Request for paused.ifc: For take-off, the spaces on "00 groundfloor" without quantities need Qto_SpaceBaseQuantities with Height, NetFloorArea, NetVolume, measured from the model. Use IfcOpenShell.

First a look at what the model holds.

```python
import ifcopenshell
import ifcopenshell.util.element
import ifcopenshell.util.unit

model = ifcopenshell.open("paused.ifc")
print(model.schema)
for unit_type in ("LENGTHUNIT", "AREAUNIT", "VOLUMEUNIT"):
    print(unit_type, ifcopenshell.util.unit.calculate_unit_scale(model, unit_type))
storey = next(s for s in model.by_type("IfcBuildingStorey") if s.Name == "00 groundfloor")
spaces = [e for e in ifcopenshell.util.element.get_decomposition(storey) if e.is_a("IfcSpace")]
for e in sorted(spaces, key=lambda e: e.id()):
    print(e.id(), e.is_a(), e.Name, list(ifcopenshell.util.element.get_psets(e, qtos_only=True)), sep=" | ")
```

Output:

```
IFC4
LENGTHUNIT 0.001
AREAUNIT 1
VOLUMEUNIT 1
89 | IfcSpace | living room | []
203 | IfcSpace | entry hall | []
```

```python
import ifcopenshell
import ifcopenshell.api.pset
import ifcopenshell.geom
import ifcopenshell.util.element
import ifcopenshell.util.shape
import ifcopenshell.util.unit

model = ifcopenshell.open("paused.ifc")
unit_scale = ifcopenshell.util.unit.calculate_unit_scale(model)
area_scale = ifcopenshell.util.unit.calculate_unit_scale(model, "AREAUNIT")
volume_scale = ifcopenshell.util.unit.calculate_unit_scale(model, "VOLUMEUNIT")
settings = ifcopenshell.geom.settings()

storey = next(s for s in model.by_type("IfcBuildingStorey") if s.Name == "00 groundfloor")
spaces = [e for e in ifcopenshell.util.element.get_decomposition(storey) if e.is_a("IfcSpace")]

for e in sorted(spaces, key=lambda e: e.id()):
    if ifcopenshell.util.element.get_psets(e, qtos_only=True, should_inherit=False):
        continue
    # Geometry comes back in metres, in the element's own axes.
    shape = ifcopenshell.geom.create_shape(settings, e)
    values = {
        "Height": ifcopenshell.util.shape.get_z(shape.geometry) / unit_scale,
        "NetFloorArea": ifcopenshell.util.shape.get_footprint_area(shape.geometry) / area_scale,
        "NetVolume": ifcopenshell.util.shape.get_volume(shape.geometry) / volume_scale,
    }
    qto = ifcopenshell.api.pset.add_qto(model, product=e, name="Qto_SpaceBaseQuantities")
    ifcopenshell.api.pset.edit_qto(model, qto=qto, properties=values)
    print(e.id(), {k: round(v, 3) for k, v in values.items()})

model.write("paused-out.ifc")
```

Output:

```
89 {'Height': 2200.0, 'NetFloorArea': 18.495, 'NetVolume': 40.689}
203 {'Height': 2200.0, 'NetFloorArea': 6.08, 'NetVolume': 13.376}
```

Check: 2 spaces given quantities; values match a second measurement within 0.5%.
